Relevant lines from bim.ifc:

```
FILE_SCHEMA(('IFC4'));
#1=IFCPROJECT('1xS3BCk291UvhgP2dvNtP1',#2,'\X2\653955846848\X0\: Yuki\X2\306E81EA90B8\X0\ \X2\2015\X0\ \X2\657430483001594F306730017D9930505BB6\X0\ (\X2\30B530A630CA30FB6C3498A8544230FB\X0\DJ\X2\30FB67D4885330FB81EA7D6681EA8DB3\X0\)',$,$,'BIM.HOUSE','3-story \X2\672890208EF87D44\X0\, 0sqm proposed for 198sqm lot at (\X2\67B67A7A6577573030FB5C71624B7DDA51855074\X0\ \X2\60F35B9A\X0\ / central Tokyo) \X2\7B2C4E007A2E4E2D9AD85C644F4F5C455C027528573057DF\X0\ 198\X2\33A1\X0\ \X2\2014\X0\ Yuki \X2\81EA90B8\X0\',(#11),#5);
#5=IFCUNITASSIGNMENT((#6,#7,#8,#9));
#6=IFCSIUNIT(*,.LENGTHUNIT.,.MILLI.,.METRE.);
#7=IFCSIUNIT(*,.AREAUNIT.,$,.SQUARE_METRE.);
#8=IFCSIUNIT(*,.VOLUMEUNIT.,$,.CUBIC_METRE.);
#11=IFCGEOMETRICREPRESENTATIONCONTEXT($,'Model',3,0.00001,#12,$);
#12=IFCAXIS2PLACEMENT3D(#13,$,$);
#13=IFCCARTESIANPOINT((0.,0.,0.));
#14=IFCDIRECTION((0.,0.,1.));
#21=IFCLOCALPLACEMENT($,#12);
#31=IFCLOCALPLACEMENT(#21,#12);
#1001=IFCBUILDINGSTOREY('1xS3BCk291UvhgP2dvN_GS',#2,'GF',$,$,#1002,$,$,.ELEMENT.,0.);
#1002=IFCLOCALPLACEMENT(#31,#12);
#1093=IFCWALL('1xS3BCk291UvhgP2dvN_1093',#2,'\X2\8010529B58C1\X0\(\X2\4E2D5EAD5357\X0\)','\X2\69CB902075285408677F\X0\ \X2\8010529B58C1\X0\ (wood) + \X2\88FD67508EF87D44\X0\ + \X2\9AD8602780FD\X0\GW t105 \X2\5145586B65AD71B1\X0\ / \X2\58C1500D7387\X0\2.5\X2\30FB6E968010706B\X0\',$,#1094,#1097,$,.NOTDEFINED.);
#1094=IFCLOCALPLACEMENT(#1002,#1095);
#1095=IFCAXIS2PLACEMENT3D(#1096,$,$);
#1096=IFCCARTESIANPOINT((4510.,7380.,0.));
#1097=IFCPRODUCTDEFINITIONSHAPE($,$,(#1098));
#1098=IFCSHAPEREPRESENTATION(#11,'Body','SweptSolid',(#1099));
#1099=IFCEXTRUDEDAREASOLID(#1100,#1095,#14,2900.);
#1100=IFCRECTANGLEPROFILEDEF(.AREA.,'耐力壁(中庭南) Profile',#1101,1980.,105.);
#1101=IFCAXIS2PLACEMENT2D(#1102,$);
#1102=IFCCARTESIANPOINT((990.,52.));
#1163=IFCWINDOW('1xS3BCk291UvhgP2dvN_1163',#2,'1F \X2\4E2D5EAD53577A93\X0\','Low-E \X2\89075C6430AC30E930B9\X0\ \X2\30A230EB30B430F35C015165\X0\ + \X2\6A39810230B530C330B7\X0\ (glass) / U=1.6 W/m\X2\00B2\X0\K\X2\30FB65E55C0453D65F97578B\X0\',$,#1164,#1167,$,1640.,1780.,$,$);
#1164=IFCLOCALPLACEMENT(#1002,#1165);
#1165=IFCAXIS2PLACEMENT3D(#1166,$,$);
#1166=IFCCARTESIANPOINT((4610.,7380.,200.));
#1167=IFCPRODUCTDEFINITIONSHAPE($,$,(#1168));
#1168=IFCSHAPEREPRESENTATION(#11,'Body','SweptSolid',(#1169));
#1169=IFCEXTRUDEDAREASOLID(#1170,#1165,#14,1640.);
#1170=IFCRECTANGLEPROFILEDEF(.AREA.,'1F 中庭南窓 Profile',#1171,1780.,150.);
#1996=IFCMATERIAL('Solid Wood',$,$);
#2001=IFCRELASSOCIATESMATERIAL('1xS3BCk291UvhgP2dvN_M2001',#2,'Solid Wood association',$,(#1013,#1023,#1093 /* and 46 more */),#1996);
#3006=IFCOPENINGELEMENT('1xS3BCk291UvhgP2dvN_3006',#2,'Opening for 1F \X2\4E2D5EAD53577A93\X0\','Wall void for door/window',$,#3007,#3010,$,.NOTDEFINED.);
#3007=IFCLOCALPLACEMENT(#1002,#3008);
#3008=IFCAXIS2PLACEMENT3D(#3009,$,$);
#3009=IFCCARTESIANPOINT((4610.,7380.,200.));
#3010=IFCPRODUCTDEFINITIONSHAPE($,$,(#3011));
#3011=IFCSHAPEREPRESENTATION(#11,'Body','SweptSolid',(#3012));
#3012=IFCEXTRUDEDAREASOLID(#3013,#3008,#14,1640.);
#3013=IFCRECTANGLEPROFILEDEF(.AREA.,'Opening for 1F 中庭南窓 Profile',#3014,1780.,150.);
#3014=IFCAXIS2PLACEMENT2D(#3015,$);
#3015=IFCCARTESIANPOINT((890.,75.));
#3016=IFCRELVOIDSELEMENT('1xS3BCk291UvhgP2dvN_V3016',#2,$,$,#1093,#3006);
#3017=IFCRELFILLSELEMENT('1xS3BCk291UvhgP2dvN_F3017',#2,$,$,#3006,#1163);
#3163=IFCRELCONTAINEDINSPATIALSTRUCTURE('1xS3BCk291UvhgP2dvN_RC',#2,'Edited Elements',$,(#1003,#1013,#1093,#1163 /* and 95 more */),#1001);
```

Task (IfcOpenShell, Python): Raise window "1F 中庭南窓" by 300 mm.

```python
import numpy as np
import ifcopenshell
import ifcopenshell.api.geometry
import ifcopenshell.util.placement
import ifcopenshell.util.unit

model = ifcopenshell.open("bim.ifc")
unit_scale = ifcopenshell.util.unit.calculate_unit_scale(model)

window = model.by_guid("1xS3BCk291UvhgP2dvN_1163")
opening = window.FillsVoids[0].RelatingOpeningElement
dz = 300.0

shift = np.array([0.0, 0.0, dz])
# The window is not placed relative to its opening, so move both.
for product in (opening, window):
    matrix = ifcopenshell.util.placement.get_local_placement(product.ObjectPlacement)
    matrix[:3, 3] += shift
    ifcopenshell.api.geometry.edit_object_placement(model, product=product, matrix=matrix, is_si=False)

print(f"moved by {dz * unit_scale:+.3f} m")

model.write("bim_rev.ifc")
```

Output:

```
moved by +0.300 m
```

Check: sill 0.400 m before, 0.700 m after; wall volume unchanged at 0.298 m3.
